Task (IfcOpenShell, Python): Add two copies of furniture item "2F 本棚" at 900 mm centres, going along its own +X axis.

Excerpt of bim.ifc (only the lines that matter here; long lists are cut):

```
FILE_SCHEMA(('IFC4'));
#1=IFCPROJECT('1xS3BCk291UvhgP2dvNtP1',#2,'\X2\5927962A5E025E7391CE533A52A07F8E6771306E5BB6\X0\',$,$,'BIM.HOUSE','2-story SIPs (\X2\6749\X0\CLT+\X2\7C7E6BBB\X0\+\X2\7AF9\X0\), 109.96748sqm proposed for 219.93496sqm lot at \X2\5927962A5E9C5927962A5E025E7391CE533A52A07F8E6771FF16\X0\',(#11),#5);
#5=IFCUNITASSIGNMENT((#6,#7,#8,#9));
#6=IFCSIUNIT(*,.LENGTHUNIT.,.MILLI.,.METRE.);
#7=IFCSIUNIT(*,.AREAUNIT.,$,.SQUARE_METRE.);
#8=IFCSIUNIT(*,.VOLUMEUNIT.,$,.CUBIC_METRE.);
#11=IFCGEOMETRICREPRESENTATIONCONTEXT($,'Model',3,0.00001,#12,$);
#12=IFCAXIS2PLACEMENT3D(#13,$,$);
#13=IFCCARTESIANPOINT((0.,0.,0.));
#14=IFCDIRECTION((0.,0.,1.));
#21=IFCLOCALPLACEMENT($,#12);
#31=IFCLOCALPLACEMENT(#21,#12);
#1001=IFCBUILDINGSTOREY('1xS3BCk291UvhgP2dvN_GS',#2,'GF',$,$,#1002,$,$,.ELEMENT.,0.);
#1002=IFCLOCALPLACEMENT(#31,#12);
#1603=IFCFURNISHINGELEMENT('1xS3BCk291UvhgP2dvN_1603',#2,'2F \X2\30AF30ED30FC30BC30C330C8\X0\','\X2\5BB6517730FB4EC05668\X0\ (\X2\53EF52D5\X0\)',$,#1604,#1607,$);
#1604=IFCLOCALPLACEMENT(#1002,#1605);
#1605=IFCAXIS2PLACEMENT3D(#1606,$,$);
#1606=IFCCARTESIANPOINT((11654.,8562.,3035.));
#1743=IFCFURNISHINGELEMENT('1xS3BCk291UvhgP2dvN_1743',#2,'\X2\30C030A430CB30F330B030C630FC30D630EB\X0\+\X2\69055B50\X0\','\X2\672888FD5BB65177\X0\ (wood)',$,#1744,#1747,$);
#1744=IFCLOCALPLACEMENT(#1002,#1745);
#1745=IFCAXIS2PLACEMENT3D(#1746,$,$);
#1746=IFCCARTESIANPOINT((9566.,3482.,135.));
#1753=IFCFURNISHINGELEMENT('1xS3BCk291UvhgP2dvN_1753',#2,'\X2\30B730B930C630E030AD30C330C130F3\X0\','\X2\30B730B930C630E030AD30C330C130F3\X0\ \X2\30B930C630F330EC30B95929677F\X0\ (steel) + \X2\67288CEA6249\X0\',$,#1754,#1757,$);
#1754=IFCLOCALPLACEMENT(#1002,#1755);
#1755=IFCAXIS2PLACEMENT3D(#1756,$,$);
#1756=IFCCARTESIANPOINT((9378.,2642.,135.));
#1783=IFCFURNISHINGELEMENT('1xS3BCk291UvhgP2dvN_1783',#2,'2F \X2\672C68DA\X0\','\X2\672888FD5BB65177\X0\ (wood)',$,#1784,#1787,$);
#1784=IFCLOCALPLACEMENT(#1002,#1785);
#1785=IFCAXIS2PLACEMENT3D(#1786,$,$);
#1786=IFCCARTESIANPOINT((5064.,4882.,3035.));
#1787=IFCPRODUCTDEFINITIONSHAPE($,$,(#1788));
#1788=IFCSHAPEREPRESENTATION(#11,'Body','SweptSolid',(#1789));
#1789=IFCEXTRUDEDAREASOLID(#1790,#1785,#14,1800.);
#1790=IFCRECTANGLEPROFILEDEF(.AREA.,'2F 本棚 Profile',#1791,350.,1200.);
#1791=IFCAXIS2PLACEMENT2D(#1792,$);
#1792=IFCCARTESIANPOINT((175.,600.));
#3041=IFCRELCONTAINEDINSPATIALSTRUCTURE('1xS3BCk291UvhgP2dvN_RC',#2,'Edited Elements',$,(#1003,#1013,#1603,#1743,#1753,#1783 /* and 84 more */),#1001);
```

```python
import ifcopenshell
import ifcopenshell.api.geometry
import ifcopenshell.api.root
import ifcopenshell.util.element
import ifcopenshell.util.placement
import ifcopenshell.util.unit

model = ifcopenshell.open("bim.ifc")
unit_scale = ifcopenshell.util.unit.calculate_unit_scale(model)


def reuse_history(source, copy):
    """copy_class also copies each property set's owner history, people and application; keep the originals."""
    for rel in copy.IsDefinedBy:
        if rel.is_a("IfcRelDefinesByProperties") and (history := rel.RelatingPropertyDefinition.OwnerHistory):
            rel.RelatingPropertyDefinition.OwnerHistory = source.OwnerHistory
            ifcopenshell.util.element.remove_deep2(model, history)


source = model.by_guid("1xS3BCk291UvhgP2dvN_1783")
base = ifcopenshell.util.placement.get_local_placement(source.ObjectPlacement)
step = base[:3, 0] * 0.9 / unit_scale

for i in range(1, 3):
    copy = ifcopenshell.api.root.copy_class(model, product=source)
    copy.Representation = ifcopenshell.util.element.copy_deep(
        model, source.Representation, exclude=["IfcGeometricRepresentationContext", "IfcRepresentationMap"]
    )
    reuse_history(source, copy)
    matrix = base.copy()
    matrix[:3, 3] += i * step
    print("added at", matrix[:3, 3].round(3) + 0.0)
    ifcopenshell.api.geometry.edit_object_placement(model, product=copy, matrix=matrix, is_si=False)

model.write("bim_updated.ifc")
```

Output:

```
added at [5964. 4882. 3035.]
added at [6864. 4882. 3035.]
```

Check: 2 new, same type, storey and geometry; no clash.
